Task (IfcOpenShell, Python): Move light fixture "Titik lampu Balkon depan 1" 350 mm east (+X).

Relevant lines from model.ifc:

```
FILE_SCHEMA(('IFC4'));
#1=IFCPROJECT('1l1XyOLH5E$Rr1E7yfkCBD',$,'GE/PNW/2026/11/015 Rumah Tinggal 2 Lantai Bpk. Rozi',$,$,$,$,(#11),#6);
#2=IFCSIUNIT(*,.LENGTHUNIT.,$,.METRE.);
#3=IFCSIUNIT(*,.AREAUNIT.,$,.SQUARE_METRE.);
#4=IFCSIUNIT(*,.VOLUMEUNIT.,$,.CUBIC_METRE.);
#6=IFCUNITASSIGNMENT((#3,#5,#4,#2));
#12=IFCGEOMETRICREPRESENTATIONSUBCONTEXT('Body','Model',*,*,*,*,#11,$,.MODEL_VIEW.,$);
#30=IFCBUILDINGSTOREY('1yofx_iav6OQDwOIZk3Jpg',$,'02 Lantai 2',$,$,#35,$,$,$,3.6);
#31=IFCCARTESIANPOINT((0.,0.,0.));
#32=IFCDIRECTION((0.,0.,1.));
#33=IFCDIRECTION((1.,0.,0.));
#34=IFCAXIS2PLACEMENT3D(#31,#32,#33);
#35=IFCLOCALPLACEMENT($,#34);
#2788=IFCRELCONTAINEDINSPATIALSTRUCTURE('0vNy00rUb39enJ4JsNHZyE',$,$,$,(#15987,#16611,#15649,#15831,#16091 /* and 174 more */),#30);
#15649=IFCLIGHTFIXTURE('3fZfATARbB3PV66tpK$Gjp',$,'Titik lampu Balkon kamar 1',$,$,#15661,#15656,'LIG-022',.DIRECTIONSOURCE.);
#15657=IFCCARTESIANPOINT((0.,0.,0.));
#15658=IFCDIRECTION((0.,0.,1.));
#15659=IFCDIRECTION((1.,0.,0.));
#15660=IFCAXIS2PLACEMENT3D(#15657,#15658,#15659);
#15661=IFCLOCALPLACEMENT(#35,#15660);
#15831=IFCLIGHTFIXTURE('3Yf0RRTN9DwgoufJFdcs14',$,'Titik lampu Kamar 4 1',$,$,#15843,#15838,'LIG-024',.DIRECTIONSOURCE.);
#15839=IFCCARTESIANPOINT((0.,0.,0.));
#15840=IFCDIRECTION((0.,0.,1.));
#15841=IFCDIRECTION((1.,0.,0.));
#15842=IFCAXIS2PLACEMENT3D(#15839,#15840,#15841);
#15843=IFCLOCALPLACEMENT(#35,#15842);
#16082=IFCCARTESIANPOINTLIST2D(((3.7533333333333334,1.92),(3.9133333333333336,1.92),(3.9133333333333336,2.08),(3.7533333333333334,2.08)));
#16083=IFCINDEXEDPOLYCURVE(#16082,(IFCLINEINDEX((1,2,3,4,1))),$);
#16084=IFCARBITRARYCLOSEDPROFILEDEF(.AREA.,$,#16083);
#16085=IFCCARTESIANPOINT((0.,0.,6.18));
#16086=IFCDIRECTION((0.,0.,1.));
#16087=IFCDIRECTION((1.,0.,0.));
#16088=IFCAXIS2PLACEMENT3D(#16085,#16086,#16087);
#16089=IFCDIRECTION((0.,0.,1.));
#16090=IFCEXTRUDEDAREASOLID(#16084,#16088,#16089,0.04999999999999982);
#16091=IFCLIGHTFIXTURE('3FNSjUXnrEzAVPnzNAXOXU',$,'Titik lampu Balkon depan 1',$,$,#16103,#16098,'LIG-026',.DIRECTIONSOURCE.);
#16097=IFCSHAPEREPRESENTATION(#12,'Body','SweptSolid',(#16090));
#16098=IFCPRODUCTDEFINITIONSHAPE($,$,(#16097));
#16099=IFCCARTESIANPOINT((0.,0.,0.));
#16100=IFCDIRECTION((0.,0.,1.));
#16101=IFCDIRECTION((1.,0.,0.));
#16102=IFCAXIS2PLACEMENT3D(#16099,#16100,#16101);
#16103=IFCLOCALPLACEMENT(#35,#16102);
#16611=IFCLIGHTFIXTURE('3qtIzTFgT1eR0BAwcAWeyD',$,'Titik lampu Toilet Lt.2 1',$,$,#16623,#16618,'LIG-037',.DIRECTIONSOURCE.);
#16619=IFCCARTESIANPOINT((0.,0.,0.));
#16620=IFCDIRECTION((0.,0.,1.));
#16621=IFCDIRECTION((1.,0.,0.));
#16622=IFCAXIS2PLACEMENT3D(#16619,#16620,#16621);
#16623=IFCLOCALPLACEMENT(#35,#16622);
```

```python
import ifcopenshell
import ifcopenshell.api.geometry
import ifcopenshell.util.placement

model = ifcopenshell.open("model.ifc")

item = model.by_guid("3FNSjUXnrEzAVPnzNAXOXU")
matrix = ifcopenshell.util.placement.get_local_placement(item.ObjectPlacement)
matrix[0, 3] += 0.35
ifcopenshell.api.geometry.edit_object_placement(model, product=item, matrix=matrix, is_si=False)

print(ifcopenshell.util.placement.get_local_placement(item.ObjectPlacement).round(3) + 0.0)

model.write("model_v2.ifc")
```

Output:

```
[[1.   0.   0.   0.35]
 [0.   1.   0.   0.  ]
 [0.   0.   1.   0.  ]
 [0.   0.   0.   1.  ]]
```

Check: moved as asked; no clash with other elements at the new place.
